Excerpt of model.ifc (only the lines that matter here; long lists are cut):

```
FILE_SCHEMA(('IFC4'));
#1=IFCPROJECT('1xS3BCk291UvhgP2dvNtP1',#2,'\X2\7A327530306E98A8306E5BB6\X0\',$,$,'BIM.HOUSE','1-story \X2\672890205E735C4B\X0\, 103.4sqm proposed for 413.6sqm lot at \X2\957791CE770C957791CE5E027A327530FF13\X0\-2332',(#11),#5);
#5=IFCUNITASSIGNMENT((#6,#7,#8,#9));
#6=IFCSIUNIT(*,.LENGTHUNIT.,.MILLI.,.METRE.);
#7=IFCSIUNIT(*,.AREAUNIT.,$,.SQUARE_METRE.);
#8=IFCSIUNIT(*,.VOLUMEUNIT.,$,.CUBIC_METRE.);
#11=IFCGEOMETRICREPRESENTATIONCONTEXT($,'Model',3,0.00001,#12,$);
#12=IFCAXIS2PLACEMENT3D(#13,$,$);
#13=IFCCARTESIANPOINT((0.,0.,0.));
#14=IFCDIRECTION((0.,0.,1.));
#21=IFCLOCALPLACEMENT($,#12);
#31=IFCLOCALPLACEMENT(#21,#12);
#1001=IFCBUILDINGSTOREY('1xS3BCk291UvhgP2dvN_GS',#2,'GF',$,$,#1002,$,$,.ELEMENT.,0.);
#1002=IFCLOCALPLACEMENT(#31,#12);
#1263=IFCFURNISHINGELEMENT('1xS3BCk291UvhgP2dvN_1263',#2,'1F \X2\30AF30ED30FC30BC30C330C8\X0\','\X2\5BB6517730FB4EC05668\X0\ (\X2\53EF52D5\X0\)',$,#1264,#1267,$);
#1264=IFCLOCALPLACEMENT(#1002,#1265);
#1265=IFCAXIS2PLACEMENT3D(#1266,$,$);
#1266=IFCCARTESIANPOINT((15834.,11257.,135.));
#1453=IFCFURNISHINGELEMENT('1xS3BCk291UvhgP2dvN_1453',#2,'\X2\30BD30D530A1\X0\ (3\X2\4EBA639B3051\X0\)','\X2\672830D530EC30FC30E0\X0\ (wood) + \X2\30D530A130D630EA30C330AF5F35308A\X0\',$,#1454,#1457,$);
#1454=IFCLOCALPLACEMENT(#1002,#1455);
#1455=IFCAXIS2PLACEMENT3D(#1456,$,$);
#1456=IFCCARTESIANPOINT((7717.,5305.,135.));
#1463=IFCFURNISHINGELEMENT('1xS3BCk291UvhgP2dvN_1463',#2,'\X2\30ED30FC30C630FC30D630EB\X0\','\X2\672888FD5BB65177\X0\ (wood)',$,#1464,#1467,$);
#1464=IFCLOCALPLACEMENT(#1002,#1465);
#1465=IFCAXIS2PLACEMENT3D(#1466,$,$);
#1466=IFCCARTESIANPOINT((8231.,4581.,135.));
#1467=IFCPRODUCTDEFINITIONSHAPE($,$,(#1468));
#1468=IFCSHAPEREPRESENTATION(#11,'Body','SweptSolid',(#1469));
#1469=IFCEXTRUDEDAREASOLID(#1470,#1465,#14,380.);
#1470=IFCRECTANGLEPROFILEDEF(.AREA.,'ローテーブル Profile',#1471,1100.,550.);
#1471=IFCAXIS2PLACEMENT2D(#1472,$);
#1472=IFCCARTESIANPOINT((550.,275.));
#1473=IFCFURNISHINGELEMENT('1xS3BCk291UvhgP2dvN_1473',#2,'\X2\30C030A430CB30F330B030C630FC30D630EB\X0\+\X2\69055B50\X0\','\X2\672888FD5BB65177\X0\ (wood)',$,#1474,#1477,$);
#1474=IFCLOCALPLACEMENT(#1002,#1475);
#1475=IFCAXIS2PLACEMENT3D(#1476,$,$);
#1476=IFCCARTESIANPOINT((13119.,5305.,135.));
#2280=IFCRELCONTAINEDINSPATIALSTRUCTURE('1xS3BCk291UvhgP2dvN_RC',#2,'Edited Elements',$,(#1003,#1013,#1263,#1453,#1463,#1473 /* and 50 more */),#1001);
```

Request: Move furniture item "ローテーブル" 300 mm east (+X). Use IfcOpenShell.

```python
import ifcopenshell
import ifcopenshell.api.geometry
import ifcopenshell.util.placement
import ifcopenshell.util.unit

model = ifcopenshell.open("model.ifc")
unit_scale = ifcopenshell.util.unit.calculate_unit_scale(model)

item = model.by_id(1463)
matrix = ifcopenshell.util.placement.get_local_placement(item.ObjectPlacement)
matrix[0, 3] += 0.3 / unit_scale
ifcopenshell.api.geometry.edit_object_placement(model, product=item, matrix=matrix, is_si=False)

print(ifcopenshell.util.placement.get_local_placement(item.ObjectPlacement).round(3) + 0.0)

model.write("model_edited.ifc")
```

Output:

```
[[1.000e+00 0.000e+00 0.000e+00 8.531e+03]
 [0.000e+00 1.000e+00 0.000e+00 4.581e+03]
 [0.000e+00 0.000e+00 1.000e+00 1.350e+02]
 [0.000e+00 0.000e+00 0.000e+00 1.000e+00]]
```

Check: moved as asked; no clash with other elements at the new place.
